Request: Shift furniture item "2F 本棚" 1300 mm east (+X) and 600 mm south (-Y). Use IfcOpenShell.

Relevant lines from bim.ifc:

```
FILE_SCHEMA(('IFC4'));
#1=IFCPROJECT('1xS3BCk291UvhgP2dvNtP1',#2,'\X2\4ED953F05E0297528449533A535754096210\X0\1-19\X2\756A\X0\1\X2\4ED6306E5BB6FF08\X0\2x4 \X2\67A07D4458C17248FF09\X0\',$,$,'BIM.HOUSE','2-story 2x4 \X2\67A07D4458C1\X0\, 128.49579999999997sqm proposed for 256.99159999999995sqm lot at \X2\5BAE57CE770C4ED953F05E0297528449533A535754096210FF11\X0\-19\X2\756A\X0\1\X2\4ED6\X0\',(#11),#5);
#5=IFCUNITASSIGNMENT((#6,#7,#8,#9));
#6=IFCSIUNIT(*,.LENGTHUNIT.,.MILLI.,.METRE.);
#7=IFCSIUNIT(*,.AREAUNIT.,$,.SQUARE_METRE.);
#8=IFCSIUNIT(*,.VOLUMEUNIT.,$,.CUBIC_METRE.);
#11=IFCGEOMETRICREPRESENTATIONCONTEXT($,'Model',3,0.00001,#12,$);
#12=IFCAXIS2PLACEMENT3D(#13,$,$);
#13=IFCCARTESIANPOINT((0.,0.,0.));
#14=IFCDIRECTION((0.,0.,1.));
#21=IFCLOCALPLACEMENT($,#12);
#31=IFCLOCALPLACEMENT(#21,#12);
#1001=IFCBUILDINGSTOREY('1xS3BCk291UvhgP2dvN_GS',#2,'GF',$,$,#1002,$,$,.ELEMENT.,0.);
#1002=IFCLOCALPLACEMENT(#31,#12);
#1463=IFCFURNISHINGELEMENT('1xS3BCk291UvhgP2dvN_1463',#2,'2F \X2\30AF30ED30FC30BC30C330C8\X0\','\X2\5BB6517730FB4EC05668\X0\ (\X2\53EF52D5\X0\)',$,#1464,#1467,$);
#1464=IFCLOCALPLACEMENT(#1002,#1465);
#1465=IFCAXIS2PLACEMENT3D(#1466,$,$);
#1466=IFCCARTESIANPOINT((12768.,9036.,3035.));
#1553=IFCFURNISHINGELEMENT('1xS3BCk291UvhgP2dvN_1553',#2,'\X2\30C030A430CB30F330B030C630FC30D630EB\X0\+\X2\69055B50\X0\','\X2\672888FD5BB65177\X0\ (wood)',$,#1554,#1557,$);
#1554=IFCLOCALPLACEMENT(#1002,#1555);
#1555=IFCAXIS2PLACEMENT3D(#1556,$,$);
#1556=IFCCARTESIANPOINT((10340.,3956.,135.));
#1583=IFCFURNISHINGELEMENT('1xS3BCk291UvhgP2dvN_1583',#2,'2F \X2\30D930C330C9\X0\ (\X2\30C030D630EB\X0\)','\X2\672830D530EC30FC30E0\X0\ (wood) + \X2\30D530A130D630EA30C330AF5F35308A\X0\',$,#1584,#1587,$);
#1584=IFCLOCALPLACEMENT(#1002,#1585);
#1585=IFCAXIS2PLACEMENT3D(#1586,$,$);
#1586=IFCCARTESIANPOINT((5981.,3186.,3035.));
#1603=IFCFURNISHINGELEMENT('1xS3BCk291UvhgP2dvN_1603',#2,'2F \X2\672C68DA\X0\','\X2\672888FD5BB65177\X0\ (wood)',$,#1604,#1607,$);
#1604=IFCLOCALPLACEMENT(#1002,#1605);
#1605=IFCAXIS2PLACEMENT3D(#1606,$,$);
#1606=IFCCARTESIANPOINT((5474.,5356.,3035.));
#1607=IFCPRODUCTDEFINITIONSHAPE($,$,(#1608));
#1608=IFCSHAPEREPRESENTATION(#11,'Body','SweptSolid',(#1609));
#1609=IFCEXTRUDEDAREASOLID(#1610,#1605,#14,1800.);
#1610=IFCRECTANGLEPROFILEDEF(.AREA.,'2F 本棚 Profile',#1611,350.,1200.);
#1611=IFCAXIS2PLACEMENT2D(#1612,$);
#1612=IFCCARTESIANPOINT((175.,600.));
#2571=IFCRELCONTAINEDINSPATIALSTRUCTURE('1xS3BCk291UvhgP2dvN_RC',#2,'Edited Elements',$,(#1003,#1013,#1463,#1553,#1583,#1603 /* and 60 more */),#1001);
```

```python
import ifcopenshell
import ifcopenshell.api.geometry
import ifcopenshell.util.placement
import ifcopenshell.util.unit

model = ifcopenshell.open("bim.ifc")
unit_scale = ifcopenshell.util.unit.calculate_unit_scale(model)

item = model.by_id(1603)
matrix = ifcopenshell.util.placement.get_local_placement(item.ObjectPlacement)
matrix[0, 3] += 1.3 / unit_scale
matrix[1, 3] -= 0.6 / unit_scale
ifcopenshell.api.geometry.edit_object_placement(model, product=item, matrix=matrix, is_si=False)

print(ifcopenshell.util.placement.get_local_placement(item.ObjectPlacement).round(3) + 0.0)

model.write("bim_edited.ifc")
```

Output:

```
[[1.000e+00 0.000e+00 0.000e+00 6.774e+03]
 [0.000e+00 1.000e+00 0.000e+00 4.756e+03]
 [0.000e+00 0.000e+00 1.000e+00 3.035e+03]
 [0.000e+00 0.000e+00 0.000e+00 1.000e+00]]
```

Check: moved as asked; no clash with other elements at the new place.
